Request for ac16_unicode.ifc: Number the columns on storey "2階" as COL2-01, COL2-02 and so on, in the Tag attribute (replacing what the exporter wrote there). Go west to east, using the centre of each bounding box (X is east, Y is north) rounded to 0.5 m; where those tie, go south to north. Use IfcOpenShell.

First a look at what the model holds.

```python
import ifcopenshell
import ifcopenshell.util.element
import ifcopenshell.util.placement

model = ifcopenshell.open("ac16_unicode.ifc")
print(model.schema)
storey = next(s for s in model.by_type("IfcBuildingStorey") if s.Name == "2階")
columns = [e for e in ifcopenshell.util.element.get_decomposition(storey) if e.is_a("IfcColumn")]
for e in sorted(columns, key=lambda e: e.id()):
    origin = ifcopenshell.util.placement.get_local_placement(e.ObjectPlacement)[:3, 3]
    print(e.id(), e.Tag, e.Name, origin.round(2) + 0.0, sep=" | ")
```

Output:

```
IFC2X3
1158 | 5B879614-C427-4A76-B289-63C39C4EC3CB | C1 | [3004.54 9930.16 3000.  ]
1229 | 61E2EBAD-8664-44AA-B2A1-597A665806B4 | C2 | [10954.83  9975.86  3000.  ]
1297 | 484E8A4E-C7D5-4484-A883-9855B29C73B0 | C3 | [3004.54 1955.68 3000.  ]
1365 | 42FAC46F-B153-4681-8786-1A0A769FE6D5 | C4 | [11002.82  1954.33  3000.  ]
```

```python
import ifcopenshell
import ifcopenshell.geom
import ifcopenshell.util.element
import ifcopenshell.util.shape

model = ifcopenshell.open("ac16_unicode.ifc")
settings = ifcopenshell.geom.settings()
settings.set("use-world-coords", True)


def centre(element):
    shape = ifcopenshell.geom.create_shape(settings, element)
    return ifcopenshell.util.shape.get_bbox_centroid(shape.geometry)


storey = next(s for s in model.by_type("IfcBuildingStorey") if s.Name == "2階")
columns = [e for e in ifcopenshell.util.element.get_decomposition(storey) if e.is_a("IfcColumn")]

# Insertion points can sit at a corner or the storey origin, so sort by the geometry (in metres).
centres = {e: centre(e) for e in columns}
columns.sort(key=lambda e: (round(centres[e][0] / 0.5), centres[e][1]))

for i, e in enumerate(columns, start=1):
    number = f"COL2-{i:02d}"
    e.Tag = number
    print(e.id(), number)

model.write("ac16_unicode_edited.ifc")
```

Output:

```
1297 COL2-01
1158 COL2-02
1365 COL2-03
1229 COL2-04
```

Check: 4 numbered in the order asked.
